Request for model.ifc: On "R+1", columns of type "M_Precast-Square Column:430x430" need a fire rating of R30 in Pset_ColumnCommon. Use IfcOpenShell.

First a look at what the model holds.

```python
import ifcopenshell
import ifcopenshell.util.element

model = ifcopenshell.open("model.ifc")
print(model.schema)
storey = next(s for s in model.by_type("IfcBuildingStorey") if s.Name == "R+1")
columns = [e for e in ifcopenshell.util.element.get_decomposition(storey) if e.is_a("IfcColumn")]
seen = {}
for e in columns:
    element_type = ifcopenshell.util.element.get_type(e)
    key = (element_type.Name if element_type != e and element_type else None, ifcopenshell.util.element.get_pset(e, "Pset_ColumnCommon", "FireRating"))
    seen[key] = seen.get(key, 0) + 1
for (name, value), count in sorted(seen.items(), key=str):
    print(count, "x", name, "|", value)
```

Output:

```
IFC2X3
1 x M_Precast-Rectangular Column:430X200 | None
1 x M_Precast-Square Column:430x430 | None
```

```python
import ifcopenshell
import ifcopenshell.api.pset
import ifcopenshell.util.element

model = ifcopenshell.open("model.ifc")

storey = next(s for s in model.by_type("IfcBuildingStorey") if s.Name == "R+1")
columns = [e for e in ifcopenshell.util.element.get_decomposition(storey) if e.is_a("IfcColumn")]

count = 0
for e in columns:
    element_type = ifcopenshell.util.element.get_type(e)
    if element_type in (None, e) or element_type.Name != "M_Precast-Square Column:430x430":
        continue
    # add_pset returns the element's existing set when there is one.
    pset = ifcopenshell.api.pset.add_pset(model, product=e, name="Pset_ColumnCommon")
    ifcopenshell.api.pset.edit_pset(model, pset=pset, properties={"FireRating": "R30"})
    count += 1

print(count, "columns updated")

model.write("model_updated.ifc")
```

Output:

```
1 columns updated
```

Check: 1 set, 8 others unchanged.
